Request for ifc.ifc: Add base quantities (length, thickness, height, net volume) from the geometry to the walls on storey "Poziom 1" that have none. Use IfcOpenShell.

First a look at what the model holds.

```python
import ifcopenshell
import ifcopenshell.util.element
import ifcopenshell.util.unit

model = ifcopenshell.open("ifc.ifc")
print(model.schema)
for unit_type in ("LENGTHUNIT", "AREAUNIT", "VOLUMEUNIT"):
    print(unit_type, ifcopenshell.util.unit.calculate_unit_scale(model, unit_type))
storey = next(s for s in model.by_type("IfcBuildingStorey") if s.Name == "Poziom 1")
walls = [e for e in ifcopenshell.util.element.get_decomposition(storey) if e.is_a("IfcWall")]
for e in sorted(walls, key=lambda e: e.id()):
    print(e.id(), e.is_a(), e.Name, list(ifcopenshell.util.element.get_psets(e, qtos_only=True)), sep=" | ")
```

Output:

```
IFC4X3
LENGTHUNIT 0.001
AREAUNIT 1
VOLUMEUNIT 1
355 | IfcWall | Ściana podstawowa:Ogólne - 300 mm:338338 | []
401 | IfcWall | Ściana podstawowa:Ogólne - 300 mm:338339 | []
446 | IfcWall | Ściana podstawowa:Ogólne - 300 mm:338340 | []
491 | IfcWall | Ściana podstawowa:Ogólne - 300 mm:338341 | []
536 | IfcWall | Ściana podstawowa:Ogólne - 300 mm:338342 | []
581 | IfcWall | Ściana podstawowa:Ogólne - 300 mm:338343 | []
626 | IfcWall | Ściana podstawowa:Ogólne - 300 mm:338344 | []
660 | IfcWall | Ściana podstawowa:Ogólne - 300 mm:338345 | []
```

```python
import ifcopenshell
import ifcopenshell.api.pset
import ifcopenshell.geom
import ifcopenshell.util.element
import ifcopenshell.util.shape
import ifcopenshell.util.unit

model = ifcopenshell.open("ifc.ifc")
unit_scale = ifcopenshell.util.unit.calculate_unit_scale(model)
volume_scale = ifcopenshell.util.unit.calculate_unit_scale(model, "VOLUMEUNIT")
settings = ifcopenshell.geom.settings()

storey = next(s for s in model.by_type("IfcBuildingStorey") if s.Name == "Poziom 1")
walls = [e for e in ifcopenshell.util.element.get_decomposition(storey) if e.is_a("IfcWall")]

for e in sorted(walls, key=lambda e: e.id()):
    if ifcopenshell.util.element.get_psets(e, qtos_only=True, should_inherit=False):
        continue
    # Geometry comes back in metres, in the element's own axes.
    shape = ifcopenshell.geom.create_shape(settings, e)
    values = {
        "Length": ifcopenshell.util.shape.get_x(shape.geometry) / unit_scale,
        "Width": ifcopenshell.util.shape.get_y(shape.geometry) / unit_scale,
        "Height": ifcopenshell.util.shape.get_z(shape.geometry) / unit_scale,
        "NetVolume": ifcopenshell.util.shape.get_volume(shape.geometry) / volume_scale,
    }
    qto = ifcopenshell.api.pset.add_qto(model, product=e, name="Qto_WallBaseQuantities")
    ifcopenshell.api.pset.edit_qto(model, qto=qto, properties=values)
    print(e.id(), {k: round(v, 3) for k, v in values.items()})

model.write("ifc_updated.ifc")
```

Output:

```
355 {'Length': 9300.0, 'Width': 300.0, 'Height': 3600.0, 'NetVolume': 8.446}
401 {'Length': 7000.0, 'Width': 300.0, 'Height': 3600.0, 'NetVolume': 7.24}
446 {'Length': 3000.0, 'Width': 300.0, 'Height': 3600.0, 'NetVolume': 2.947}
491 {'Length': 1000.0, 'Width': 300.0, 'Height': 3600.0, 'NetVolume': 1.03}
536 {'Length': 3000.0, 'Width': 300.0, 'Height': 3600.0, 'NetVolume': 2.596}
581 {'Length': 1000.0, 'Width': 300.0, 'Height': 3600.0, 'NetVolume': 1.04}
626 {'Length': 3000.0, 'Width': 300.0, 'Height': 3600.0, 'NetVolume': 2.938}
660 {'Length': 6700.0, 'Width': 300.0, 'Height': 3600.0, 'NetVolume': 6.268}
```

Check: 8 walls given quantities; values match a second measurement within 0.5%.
